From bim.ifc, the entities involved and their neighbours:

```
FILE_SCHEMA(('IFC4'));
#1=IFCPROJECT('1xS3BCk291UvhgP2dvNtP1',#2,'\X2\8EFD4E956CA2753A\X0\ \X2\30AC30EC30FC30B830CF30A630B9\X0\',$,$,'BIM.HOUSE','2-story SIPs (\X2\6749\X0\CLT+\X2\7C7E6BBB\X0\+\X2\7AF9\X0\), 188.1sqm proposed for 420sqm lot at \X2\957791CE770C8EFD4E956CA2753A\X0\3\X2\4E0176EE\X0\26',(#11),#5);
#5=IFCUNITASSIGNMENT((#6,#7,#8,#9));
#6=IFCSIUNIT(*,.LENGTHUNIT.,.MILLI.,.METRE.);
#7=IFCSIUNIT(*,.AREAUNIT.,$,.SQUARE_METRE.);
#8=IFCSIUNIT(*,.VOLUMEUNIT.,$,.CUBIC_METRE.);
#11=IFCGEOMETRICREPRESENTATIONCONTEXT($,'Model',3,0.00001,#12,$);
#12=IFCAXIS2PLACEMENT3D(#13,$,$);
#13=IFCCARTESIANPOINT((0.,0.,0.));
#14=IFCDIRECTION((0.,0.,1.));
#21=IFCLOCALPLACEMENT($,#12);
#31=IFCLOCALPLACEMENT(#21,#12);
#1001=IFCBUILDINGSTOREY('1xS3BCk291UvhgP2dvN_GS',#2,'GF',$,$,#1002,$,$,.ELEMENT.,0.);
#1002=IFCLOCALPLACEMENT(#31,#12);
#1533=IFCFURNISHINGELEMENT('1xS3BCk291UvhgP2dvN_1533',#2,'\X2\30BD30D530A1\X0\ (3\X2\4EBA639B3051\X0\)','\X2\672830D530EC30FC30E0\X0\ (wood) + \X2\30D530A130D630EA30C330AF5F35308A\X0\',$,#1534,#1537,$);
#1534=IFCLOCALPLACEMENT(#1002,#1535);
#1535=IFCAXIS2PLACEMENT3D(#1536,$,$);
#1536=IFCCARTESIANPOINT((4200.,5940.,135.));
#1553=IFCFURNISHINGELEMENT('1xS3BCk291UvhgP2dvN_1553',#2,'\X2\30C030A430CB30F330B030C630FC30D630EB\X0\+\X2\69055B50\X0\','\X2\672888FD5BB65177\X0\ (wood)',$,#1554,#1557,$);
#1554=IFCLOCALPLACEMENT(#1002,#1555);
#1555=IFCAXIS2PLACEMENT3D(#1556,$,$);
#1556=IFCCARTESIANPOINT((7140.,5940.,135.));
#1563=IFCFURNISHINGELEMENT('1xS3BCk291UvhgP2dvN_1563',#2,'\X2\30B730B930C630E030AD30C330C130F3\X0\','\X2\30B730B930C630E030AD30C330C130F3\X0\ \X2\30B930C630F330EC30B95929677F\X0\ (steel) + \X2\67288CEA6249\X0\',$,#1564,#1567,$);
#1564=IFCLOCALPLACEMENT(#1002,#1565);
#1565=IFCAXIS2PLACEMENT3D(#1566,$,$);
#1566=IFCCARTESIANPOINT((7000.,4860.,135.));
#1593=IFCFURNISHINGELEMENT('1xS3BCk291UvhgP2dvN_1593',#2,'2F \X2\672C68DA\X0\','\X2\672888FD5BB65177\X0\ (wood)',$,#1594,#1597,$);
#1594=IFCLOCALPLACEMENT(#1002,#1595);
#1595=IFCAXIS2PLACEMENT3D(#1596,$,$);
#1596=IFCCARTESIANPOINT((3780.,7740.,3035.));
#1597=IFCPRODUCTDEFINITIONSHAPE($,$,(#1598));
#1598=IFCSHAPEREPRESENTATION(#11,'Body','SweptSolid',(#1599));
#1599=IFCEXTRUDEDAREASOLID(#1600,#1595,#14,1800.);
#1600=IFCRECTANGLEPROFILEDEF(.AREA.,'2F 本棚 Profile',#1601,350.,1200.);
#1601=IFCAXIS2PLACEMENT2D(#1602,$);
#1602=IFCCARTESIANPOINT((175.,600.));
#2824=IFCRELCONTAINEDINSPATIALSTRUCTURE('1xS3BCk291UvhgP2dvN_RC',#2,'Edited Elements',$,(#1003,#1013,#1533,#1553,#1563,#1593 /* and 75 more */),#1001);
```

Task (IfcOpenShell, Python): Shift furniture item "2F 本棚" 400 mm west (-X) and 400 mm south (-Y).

```python
import ifcopenshell
import ifcopenshell.api.geometry
import ifcopenshell.util.placement
import ifcopenshell.util.unit

model = ifcopenshell.open("bim.ifc")
unit_scale = ifcopenshell.util.unit.calculate_unit_scale(model)

item = model.by_guid("1xS3BCk291UvhgP2dvN_1593")
matrix = ifcopenshell.util.placement.get_local_placement(item.ObjectPlacement)
matrix[0, 3] -= 0.4 / unit_scale
matrix[1, 3] -= 0.4 / unit_scale
ifcopenshell.api.geometry.edit_object_placement(model, product=item, matrix=matrix, is_si=False)

print(ifcopenshell.util.placement.get_local_placement(item.ObjectPlacement).round(3) + 0.0)

model.write("bim_rev.ifc")
```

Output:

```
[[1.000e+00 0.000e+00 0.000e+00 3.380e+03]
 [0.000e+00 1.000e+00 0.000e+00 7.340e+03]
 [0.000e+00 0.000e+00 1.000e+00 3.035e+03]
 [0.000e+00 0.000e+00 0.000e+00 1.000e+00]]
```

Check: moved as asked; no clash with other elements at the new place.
